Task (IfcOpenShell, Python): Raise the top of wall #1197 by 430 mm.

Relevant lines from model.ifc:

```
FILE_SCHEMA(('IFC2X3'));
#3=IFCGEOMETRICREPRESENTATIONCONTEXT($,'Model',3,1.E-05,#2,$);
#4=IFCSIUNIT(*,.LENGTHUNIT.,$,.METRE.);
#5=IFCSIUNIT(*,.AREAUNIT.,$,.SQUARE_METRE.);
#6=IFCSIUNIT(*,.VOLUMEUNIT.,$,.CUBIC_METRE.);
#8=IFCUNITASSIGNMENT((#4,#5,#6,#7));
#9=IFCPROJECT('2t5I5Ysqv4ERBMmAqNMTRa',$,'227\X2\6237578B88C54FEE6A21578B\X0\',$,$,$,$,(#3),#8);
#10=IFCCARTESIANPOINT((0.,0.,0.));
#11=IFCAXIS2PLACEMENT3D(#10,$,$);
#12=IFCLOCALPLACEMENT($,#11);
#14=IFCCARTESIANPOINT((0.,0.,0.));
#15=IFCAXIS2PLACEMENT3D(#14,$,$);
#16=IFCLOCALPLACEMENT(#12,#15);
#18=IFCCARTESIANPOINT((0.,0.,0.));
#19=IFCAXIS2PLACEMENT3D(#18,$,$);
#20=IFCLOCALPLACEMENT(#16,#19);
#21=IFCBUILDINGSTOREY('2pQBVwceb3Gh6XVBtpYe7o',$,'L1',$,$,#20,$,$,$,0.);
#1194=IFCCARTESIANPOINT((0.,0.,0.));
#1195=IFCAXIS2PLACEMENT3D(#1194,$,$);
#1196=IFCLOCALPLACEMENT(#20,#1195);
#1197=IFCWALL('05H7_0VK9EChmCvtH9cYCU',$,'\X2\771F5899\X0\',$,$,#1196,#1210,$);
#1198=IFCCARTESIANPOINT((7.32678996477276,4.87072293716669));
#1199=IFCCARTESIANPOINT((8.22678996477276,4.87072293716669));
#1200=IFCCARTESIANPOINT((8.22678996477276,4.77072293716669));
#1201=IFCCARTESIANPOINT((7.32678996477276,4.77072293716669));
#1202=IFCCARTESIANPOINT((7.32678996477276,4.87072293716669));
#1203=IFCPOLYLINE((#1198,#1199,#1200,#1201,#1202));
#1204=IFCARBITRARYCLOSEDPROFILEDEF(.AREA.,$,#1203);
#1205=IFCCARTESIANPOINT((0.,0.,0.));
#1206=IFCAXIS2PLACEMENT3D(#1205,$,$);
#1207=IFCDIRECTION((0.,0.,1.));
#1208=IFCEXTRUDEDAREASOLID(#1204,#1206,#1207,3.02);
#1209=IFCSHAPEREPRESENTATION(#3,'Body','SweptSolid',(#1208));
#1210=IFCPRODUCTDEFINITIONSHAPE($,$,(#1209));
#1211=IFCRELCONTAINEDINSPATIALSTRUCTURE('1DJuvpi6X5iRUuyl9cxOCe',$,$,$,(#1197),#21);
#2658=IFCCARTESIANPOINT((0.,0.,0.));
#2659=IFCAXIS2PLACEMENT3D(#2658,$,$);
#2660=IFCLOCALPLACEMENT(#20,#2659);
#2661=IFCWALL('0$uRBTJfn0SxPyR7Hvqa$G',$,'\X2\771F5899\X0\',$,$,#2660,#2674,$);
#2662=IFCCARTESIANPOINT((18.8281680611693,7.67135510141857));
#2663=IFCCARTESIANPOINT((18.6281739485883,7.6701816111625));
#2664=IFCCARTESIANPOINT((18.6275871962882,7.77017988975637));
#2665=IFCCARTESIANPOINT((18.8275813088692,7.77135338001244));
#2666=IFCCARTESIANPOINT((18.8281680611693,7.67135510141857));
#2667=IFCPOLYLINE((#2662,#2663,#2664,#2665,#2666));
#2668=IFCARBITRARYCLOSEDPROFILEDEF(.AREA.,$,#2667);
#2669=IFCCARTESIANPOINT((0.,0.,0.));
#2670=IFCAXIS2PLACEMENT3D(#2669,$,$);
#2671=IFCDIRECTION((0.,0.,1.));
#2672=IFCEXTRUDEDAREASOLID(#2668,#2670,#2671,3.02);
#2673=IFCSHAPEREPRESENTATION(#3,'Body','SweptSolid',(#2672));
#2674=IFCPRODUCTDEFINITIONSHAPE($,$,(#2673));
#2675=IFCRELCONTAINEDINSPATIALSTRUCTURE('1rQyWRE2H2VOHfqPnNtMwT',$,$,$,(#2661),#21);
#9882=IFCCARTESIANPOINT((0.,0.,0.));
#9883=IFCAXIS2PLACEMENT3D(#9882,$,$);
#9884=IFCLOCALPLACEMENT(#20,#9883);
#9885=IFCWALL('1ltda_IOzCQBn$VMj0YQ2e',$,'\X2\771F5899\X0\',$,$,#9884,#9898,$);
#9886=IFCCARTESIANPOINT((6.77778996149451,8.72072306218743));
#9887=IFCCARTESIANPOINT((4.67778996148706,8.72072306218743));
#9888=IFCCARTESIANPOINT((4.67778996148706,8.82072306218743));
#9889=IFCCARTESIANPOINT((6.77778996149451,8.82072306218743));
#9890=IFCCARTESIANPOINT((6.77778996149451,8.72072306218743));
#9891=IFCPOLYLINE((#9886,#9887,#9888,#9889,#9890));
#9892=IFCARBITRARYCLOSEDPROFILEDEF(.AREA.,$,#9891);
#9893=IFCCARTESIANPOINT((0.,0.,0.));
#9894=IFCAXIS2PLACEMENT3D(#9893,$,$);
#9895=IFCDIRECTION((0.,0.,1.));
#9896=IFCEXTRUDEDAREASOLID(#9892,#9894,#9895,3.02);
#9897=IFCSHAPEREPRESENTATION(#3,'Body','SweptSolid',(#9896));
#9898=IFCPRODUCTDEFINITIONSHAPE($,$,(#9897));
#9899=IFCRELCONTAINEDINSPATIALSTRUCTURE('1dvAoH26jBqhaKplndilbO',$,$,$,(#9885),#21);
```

```python
import ifcopenshell
import ifcopenshell.geom
import ifcopenshell.util.shape

model = ifcopenshell.open("model.ifc")
settings = ifcopenshell.geom.settings()


def volume(element):
    """Net volume in cubic metres, openings subtracted."""
    shape = ifcopenshell.geom.create_shape(settings, element)
    return ifcopenshell.util.shape.get_volume(shape.geometry)


wall = model.by_guid("05H7_0VK9EChmCvtH9cYCU")
before = volume(wall)

body = next(r for r in wall.Representation.Representations if r.RepresentationIdentifier == "Body")
solid = body.Items[0]
old_height = solid.Depth
solid.Depth += 0.43
after = volume(wall)

print(f"height {old_height:g} -> {solid.Depth:g}, volume {before:.3f} -> {after:.3f} m3")

model.write("model_rev.ifc")
```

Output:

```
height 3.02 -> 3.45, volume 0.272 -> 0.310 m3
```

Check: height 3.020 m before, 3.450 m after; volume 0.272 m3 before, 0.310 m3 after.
